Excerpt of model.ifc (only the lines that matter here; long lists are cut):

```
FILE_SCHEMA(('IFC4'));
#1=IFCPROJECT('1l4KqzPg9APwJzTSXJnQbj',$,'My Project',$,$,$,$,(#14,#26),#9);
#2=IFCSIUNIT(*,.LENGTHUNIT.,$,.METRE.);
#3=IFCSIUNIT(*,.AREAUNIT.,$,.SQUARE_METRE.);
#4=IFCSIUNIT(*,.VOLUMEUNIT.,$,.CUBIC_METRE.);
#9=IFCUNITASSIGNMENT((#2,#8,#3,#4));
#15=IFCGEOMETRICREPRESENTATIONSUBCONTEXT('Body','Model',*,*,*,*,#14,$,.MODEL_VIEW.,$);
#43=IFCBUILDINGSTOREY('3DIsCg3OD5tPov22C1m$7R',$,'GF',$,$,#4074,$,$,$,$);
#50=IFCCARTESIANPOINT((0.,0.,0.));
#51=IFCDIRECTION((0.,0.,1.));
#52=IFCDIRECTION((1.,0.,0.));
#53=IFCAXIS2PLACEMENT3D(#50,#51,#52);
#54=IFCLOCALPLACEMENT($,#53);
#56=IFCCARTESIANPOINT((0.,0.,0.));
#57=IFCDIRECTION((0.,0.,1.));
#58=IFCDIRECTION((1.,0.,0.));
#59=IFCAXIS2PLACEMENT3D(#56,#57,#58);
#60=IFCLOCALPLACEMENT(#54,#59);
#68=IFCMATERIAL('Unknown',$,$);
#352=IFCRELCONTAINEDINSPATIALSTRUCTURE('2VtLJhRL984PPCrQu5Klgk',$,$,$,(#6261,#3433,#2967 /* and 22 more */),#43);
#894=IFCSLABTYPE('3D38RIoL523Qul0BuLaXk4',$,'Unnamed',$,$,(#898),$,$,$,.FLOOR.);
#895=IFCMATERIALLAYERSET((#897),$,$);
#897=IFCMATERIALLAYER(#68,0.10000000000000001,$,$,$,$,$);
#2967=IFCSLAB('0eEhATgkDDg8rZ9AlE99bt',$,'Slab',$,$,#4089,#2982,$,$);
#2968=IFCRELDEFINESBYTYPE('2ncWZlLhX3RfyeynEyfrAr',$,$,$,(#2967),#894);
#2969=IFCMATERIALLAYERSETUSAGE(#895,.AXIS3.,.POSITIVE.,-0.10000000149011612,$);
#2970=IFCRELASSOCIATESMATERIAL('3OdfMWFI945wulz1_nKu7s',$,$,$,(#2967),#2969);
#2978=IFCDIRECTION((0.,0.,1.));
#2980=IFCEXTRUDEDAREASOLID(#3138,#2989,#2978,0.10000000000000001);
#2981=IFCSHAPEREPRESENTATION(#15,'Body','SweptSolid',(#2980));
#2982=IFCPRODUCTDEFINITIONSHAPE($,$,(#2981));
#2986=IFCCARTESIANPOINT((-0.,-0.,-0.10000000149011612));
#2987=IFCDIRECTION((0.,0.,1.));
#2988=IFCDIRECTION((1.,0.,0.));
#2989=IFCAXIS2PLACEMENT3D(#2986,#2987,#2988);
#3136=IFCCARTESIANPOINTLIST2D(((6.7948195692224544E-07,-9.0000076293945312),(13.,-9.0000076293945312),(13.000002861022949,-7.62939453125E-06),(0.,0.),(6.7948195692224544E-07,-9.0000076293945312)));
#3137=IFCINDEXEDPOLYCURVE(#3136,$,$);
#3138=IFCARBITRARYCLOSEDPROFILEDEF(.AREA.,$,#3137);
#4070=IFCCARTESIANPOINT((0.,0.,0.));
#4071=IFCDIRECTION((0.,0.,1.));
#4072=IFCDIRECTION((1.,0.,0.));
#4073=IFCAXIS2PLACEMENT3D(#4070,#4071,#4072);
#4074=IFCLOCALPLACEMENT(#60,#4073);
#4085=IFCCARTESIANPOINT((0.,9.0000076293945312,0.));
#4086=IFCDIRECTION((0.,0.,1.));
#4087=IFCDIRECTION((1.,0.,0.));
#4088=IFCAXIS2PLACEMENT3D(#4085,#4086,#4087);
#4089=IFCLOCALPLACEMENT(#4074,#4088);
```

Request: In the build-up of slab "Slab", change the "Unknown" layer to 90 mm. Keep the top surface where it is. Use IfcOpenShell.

```python
import ifcopenshell
import ifcopenshell.util.element
import ifcopenshell.util.representation
import ifcopenshell.util.unit

model = ifcopenshell.open("model.ifc")
unit_scale = ifcopenshell.util.unit.calculate_unit_scale(model)

layer_set = model.by_id(895)
layer = next(l for l in layer_set.MaterialLayers if l.Material and l.Material.Name == "Unknown")
change = 0.09 / unit_scale - layer.LayerThickness
layer.LayerThickness += change

# Geometry does not follow the layer set by itself.
slabs = [e for e in ifcopenshell.util.element.get_elements_by_material(model, layer_set) if e.is_a("IfcSlab")]
for slab in sorted(slabs, key=lambda e: e.id()):
    body = ifcopenshell.util.representation.get_representation(slab, "Model", "Body")
    solid = body.Items[0]
    old_depth = solid.Depth
    solid.Depth += change
    # Extruded upwards: lower the start of the extrusion so the top stays.
    x, y, z = solid.Position.Location.Coordinates
    solid.Position.Location = model.createIfcCartesianPoint((x, y, z - change))
    print(slab.id(), f"{old_depth:g} -> {solid.Depth:g}")

# The layers are counted up from the underside, which has moved.
for usage in {ifcopenshell.util.element.get_material(slab) for slab in slabs}:
    usage.OffsetFromReferenceLine -= change

model.write("model_v2.ifc")
```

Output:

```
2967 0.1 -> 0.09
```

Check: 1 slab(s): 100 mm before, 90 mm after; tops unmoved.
